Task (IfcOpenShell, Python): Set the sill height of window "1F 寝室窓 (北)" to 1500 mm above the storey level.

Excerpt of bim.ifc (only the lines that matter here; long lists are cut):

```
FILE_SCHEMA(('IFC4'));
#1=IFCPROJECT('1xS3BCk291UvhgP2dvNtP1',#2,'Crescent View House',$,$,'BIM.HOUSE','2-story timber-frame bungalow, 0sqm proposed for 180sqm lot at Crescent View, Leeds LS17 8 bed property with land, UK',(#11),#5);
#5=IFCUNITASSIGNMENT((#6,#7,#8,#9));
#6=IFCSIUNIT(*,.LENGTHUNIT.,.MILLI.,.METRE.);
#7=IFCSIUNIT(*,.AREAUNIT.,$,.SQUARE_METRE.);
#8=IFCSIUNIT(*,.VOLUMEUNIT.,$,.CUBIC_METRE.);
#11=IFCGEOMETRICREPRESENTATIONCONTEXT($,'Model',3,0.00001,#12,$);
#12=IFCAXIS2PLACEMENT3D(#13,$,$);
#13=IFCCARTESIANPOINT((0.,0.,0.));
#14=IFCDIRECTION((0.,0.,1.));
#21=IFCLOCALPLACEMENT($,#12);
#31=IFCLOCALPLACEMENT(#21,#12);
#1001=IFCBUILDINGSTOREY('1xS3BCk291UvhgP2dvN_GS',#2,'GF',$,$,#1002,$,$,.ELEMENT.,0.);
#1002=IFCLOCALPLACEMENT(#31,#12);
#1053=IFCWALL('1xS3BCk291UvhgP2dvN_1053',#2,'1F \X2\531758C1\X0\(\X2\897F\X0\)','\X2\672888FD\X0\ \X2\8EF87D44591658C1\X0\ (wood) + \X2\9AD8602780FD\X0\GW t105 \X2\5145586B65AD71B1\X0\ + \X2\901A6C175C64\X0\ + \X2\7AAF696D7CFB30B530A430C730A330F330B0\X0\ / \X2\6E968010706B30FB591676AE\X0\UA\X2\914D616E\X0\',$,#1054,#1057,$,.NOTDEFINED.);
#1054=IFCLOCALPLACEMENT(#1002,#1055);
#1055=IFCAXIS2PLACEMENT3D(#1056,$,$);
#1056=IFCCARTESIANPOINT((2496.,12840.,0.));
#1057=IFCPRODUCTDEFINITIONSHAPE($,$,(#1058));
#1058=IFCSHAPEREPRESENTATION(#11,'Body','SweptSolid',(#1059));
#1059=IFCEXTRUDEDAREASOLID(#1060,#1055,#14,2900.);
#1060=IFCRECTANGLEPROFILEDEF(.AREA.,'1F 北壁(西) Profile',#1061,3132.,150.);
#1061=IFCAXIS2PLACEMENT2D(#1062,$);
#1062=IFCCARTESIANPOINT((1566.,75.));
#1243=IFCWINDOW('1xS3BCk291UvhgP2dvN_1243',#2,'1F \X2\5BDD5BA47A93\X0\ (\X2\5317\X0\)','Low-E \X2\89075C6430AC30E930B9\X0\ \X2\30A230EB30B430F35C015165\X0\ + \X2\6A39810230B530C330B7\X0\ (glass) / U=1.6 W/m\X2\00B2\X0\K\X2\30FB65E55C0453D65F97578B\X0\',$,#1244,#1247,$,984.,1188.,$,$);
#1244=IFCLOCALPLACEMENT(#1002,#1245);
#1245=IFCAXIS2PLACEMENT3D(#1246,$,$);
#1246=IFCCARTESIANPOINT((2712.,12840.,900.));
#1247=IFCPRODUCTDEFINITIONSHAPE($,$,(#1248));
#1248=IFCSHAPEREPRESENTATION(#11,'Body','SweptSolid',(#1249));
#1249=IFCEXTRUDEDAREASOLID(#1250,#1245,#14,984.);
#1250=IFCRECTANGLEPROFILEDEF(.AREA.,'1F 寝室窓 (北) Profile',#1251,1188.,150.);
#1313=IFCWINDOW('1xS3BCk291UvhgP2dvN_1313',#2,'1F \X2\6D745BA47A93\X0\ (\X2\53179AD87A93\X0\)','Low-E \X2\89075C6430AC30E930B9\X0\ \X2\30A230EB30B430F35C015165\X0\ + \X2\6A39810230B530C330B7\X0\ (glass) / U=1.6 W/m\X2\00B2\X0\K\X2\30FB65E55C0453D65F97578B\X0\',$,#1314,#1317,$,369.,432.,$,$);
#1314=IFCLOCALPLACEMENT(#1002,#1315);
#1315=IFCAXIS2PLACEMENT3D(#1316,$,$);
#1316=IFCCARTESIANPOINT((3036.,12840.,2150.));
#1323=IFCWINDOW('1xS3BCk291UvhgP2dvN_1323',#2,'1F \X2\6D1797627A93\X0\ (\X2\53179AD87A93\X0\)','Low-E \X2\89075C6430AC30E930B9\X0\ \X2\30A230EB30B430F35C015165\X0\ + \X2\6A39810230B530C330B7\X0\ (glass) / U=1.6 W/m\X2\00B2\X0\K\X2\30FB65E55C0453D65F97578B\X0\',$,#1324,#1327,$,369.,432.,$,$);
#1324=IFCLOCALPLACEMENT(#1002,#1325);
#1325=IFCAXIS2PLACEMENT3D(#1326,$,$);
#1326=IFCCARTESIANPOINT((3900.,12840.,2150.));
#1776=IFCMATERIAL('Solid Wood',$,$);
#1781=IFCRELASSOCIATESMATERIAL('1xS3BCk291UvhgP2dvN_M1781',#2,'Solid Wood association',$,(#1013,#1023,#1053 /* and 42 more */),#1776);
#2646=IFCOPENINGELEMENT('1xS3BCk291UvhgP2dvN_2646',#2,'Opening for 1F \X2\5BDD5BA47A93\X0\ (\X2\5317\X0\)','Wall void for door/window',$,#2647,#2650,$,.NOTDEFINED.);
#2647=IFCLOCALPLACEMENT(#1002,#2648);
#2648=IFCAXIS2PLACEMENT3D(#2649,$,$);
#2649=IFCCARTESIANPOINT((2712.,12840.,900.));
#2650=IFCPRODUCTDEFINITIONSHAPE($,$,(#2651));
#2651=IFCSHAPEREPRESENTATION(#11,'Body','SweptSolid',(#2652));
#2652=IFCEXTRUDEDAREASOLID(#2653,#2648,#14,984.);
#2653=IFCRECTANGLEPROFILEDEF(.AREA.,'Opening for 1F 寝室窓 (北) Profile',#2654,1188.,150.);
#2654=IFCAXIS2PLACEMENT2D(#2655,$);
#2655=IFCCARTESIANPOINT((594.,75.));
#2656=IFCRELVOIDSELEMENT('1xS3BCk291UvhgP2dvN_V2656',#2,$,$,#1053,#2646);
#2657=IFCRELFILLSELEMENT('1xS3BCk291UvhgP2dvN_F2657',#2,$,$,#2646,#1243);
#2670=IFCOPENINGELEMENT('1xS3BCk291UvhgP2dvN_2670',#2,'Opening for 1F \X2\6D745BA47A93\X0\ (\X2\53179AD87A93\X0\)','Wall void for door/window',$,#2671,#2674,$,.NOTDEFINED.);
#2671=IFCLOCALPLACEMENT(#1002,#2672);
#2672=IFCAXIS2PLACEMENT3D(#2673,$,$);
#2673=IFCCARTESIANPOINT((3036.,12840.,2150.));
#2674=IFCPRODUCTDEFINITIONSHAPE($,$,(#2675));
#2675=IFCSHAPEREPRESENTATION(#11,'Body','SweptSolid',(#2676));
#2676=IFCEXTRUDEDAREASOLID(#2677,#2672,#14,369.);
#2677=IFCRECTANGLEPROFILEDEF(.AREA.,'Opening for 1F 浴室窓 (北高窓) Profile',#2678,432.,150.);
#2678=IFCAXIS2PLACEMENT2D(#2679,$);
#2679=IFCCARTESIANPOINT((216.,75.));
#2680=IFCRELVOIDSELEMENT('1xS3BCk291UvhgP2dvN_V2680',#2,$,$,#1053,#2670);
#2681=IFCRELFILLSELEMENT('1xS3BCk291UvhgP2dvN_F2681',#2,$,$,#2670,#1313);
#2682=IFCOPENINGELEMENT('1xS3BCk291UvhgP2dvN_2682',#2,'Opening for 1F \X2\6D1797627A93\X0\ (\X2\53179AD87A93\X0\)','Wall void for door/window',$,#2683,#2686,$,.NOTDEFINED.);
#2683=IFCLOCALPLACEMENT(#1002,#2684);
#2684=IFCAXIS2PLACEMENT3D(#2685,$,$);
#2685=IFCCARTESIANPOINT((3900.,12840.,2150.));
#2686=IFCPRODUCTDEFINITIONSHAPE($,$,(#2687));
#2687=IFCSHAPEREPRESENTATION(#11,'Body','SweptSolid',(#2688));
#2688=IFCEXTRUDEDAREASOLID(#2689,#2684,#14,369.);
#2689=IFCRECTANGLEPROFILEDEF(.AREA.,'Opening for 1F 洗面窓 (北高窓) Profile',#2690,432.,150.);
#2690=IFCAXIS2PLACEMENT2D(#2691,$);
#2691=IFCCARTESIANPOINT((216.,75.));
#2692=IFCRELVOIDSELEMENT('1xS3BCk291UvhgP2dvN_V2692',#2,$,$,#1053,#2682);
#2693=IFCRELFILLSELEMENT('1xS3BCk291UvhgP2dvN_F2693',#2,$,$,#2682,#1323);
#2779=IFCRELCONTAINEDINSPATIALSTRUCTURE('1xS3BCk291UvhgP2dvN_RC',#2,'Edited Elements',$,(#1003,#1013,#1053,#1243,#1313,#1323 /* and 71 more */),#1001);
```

```python
import numpy as np
import ifcopenshell
import ifcopenshell.api.geometry
import ifcopenshell.geom
import ifcopenshell.util.element
import ifcopenshell.util.placement
import ifcopenshell.util.shape
import ifcopenshell.util.unit

model = ifcopenshell.open("bim.ifc")
unit_scale = ifcopenshell.util.unit.calculate_unit_scale(model)

window = model.by_guid("1xS3BCk291UvhgP2dvN_1243")
opening = window.FillsVoids[0].RelatingOpeningElement
storey = ifcopenshell.util.element.get_container(window, ifc_class="IfcBuildingStorey")
level = ifcopenshell.util.placement.get_local_placement(storey.ObjectPlacement)[2, 3]

# The opening's origin need not be at the sill, so measure its lowest point.
shape = ifcopenshell.geom.create_shape(ifcopenshell.geom.settings(), opening)
bottom = ifcopenshell.util.shape.get_shape_bottom_elevation(shape, shape.geometry) / unit_scale
dz = level + 1500.0 - bottom

shift = np.array([0.0, 0.0, dz])
# The window is not placed relative to its opening, so move both.
for product in (opening, window):
    matrix = ifcopenshell.util.placement.get_local_placement(product.ObjectPlacement)
    matrix[:3, 3] += shift
    ifcopenshell.api.geometry.edit_object_placement(model, product=product, matrix=matrix, is_si=False)

print(f"moved by {dz * unit_scale:+.3f} m")

model.write("bim-out.ifc")
```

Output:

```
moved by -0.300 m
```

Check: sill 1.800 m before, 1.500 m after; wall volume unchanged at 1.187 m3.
